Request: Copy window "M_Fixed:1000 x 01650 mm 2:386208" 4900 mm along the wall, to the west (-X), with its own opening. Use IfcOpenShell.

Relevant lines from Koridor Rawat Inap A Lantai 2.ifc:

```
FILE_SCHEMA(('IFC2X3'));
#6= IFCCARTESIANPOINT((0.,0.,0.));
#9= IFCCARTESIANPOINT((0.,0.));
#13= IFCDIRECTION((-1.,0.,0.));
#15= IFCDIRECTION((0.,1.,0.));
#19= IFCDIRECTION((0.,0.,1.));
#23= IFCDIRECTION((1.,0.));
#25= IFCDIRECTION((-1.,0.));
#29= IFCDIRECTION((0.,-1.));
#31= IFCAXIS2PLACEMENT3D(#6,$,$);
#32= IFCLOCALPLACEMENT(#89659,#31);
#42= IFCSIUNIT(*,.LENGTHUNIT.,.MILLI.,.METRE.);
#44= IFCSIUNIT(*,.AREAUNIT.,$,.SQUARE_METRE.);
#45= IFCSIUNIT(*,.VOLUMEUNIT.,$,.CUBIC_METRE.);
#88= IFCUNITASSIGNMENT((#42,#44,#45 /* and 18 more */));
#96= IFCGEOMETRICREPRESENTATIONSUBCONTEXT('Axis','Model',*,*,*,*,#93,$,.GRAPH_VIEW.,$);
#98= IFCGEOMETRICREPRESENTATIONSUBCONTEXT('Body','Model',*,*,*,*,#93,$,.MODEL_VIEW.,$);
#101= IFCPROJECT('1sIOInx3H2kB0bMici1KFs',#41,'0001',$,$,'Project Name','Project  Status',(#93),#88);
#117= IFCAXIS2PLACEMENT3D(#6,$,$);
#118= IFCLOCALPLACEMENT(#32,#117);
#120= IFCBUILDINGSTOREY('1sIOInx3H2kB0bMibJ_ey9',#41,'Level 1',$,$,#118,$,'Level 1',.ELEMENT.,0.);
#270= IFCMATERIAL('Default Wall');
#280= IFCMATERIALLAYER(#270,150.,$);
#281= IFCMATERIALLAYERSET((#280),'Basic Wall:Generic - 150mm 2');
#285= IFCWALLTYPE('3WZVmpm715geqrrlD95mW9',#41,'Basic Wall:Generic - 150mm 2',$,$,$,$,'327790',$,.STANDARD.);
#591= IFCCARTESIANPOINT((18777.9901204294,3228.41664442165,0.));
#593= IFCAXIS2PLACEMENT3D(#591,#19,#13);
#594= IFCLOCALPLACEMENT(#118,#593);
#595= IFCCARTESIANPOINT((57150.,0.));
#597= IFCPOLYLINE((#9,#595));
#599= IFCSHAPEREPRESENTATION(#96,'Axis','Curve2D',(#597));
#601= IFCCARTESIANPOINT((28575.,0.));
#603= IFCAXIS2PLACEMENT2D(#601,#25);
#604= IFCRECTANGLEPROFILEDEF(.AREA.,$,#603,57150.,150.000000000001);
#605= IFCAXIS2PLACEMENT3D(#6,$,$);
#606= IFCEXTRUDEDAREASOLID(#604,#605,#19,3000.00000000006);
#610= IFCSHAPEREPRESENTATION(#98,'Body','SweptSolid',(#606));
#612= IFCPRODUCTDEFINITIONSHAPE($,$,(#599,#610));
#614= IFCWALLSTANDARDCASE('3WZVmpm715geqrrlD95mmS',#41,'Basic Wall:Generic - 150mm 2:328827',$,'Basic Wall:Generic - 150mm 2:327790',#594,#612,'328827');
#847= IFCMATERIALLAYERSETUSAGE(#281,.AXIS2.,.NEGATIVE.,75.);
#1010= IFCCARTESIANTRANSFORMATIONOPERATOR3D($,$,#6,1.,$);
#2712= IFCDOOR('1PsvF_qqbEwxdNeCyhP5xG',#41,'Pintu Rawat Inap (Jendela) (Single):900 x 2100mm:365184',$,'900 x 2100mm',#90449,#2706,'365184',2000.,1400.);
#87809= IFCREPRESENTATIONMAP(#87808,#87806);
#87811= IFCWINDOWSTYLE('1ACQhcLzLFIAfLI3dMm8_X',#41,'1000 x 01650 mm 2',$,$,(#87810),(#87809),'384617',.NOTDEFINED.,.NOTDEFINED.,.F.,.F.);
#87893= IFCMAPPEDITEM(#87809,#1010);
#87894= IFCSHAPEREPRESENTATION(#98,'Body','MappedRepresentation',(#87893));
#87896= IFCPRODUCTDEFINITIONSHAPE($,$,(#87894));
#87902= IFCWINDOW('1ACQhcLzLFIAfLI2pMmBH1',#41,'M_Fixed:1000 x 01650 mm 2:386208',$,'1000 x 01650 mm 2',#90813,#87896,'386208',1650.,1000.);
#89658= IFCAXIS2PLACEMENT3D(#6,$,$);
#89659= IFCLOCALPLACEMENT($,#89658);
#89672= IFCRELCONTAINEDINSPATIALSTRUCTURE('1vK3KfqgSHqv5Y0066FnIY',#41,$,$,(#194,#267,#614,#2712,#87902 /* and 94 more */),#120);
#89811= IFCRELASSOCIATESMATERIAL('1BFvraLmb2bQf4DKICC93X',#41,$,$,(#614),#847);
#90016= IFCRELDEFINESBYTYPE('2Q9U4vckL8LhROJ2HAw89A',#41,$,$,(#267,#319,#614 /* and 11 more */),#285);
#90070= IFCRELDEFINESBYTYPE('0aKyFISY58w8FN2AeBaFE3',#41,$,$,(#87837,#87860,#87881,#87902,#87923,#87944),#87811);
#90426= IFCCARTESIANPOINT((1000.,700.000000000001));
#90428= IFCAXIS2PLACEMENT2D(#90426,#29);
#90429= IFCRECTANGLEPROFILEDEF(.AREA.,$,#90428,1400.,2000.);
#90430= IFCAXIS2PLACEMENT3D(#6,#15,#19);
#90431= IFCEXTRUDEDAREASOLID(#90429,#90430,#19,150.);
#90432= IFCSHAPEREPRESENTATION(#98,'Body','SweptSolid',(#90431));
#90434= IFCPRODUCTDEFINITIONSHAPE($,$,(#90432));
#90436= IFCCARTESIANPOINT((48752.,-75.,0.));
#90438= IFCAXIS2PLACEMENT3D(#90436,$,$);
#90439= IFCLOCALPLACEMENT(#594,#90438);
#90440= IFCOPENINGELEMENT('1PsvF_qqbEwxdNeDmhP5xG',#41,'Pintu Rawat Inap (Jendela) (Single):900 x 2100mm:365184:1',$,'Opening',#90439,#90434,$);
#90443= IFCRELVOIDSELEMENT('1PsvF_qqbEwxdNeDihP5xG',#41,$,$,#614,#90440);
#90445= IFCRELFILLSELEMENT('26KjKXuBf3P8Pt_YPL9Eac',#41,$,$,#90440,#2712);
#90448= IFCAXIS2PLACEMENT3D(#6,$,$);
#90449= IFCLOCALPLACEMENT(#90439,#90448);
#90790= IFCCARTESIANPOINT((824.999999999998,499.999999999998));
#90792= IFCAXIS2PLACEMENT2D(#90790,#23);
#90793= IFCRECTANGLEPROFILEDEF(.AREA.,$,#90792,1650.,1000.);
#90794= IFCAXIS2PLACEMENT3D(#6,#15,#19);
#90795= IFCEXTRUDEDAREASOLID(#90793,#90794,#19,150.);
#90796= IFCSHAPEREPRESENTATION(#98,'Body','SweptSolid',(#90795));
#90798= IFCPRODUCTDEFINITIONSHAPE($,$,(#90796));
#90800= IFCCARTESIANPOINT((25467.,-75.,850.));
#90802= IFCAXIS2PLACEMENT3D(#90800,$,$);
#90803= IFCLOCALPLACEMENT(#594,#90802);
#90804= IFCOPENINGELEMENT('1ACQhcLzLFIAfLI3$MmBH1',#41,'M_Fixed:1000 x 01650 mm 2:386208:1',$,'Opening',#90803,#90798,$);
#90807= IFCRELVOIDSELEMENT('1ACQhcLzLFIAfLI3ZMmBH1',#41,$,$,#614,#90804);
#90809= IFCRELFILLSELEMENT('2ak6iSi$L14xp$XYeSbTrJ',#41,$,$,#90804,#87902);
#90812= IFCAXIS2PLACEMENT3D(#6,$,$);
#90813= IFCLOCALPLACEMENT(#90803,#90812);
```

```python
import ifcopenshell
import ifcopenshell.api.feature
import ifcopenshell.api.geometry
import ifcopenshell.api.root
import ifcopenshell.geom
import ifcopenshell.util.element
import ifcopenshell.util.placement
import ifcopenshell.util.shape
import ifcopenshell.util.unit

model = ifcopenshell.open("Koridor Rawat Inap A Lantai 2.ifc")
unit_scale = ifcopenshell.util.unit.calculate_unit_scale(model)
settings = ifcopenshell.geom.settings()


def volume(element):
    """Net volume in cubic metres, openings subtracted."""
    shape = ifcopenshell.geom.create_shape(settings, element)
    return ifcopenshell.util.shape.get_volume(shape.geometry)


def reuse_history(source, copy):
    """copy_class also copies each property set's owner history, people and application; keep the originals."""
    for rel in copy.IsDefinedBy:
        if rel.is_a("IfcRelDefinesByProperties") and (history := rel.RelatingPropertyDefinition.OwnerHistory):
            rel.RelatingPropertyDefinition.OwnerHistory = source.OwnerHistory
            ifcopenshell.util.element.remove_deep2(model, history)


window = model.by_guid("1ACQhcLzLFIAfLI2pMmBH1")
opening = window.FillsVoids[0].RelatingOpeningElement
wall = opening.VoidsElements[0].RelatingBuildingElement
before = volume(wall)
shift = ifcopenshell.util.placement.get_local_placement(wall.ObjectPlacement)[:3, 0] * 4.9 / unit_scale

# copy_class copies the void relationship, type, container and properties, but no geometry.
new_opening = ifcopenshell.api.root.copy_class(model, product=opening)
new_opening.Representation = ifcopenshell.util.element.copy_deep(
    model, opening.Representation, exclude=["IfcGeometricRepresentationContext", "IfcRepresentationMap"]
)
new_opening.Name = "M_Fixed:1000 x 01650 mm 2"
new_window = ifcopenshell.api.root.copy_class(model, product=window)
new_window.Representation = ifcopenshell.util.element.copy_deep(
    model, window.Representation, exclude=["IfcGeometricRepresentationContext", "IfcRepresentationMap"]
)
new_window.Name = "M_Fixed:1000 x 01650 mm 2"
new_window.Tag = None
reuse_history(window, new_window)
fills = ifcopenshell.api.feature.add_filling(model, opening=new_opening, element=new_window)
fills.OwnerHistory = new_window.OwnerHistory  # required in IFC2X3

for old, new in ((opening, new_opening), (window, new_window)):
    matrix = ifcopenshell.util.placement.get_local_placement(old.ObjectPlacement)
    matrix[:3, 3] += shift
    ifcopenshell.api.geometry.edit_object_placement(model, product=new, matrix=matrix, is_si=False)

after = volume(wall)

print(f"wall volume {before:.3f} -> {after:.3f} m3")

model.write("Koridor Rawat Inap A Lantai 2-out.ifc")
```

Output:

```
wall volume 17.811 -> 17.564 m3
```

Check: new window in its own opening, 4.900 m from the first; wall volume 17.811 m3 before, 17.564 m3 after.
